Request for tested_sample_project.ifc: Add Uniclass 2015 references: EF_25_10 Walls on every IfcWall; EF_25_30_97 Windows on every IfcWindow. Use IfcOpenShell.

First a look at what the model holds.

```python
import ifcopenshell

model = ifcopenshell.open("tested_sample_project.ifc")
print(model.schema)
print("classifications:", [c.Name for c in model.by_type("IfcClassification")])
for ifc_class in ("IfcDoor", "IfcRoof", "IfcStair", "IfcWall", "IfcWindow"):
    print(ifc_class, len(model.by_type(ifc_class)))
```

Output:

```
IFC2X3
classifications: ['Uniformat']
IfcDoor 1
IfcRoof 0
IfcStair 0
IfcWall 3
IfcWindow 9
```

```python
import ifcopenshell
import ifcopenshell.api.classification

model = ifcopenshell.open("tested_sample_project.ifc")

# IFC2X3 requires Source and Edition and has no link from the project to the system.
system = model.create_entity("IfcClassification", Source="NBS", Edition="2015", Name="Uniclass 2015")

codes = {
    "IfcWall": ("EF_25_10", "Walls"),
    "IfcWindow": ("EF_25_30_97", "Windows"),
}
for ifc_class, (code, name) in codes.items():
    products = model.by_type(ifc_class)
    ifcopenshell.api.classification.add_reference(
        model, products=products, classification=system, identification=code, name=name
    )
    print(code, len(products))

model.write("tested_sample_project_v2.ifc")
```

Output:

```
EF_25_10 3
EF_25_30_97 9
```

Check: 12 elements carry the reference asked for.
